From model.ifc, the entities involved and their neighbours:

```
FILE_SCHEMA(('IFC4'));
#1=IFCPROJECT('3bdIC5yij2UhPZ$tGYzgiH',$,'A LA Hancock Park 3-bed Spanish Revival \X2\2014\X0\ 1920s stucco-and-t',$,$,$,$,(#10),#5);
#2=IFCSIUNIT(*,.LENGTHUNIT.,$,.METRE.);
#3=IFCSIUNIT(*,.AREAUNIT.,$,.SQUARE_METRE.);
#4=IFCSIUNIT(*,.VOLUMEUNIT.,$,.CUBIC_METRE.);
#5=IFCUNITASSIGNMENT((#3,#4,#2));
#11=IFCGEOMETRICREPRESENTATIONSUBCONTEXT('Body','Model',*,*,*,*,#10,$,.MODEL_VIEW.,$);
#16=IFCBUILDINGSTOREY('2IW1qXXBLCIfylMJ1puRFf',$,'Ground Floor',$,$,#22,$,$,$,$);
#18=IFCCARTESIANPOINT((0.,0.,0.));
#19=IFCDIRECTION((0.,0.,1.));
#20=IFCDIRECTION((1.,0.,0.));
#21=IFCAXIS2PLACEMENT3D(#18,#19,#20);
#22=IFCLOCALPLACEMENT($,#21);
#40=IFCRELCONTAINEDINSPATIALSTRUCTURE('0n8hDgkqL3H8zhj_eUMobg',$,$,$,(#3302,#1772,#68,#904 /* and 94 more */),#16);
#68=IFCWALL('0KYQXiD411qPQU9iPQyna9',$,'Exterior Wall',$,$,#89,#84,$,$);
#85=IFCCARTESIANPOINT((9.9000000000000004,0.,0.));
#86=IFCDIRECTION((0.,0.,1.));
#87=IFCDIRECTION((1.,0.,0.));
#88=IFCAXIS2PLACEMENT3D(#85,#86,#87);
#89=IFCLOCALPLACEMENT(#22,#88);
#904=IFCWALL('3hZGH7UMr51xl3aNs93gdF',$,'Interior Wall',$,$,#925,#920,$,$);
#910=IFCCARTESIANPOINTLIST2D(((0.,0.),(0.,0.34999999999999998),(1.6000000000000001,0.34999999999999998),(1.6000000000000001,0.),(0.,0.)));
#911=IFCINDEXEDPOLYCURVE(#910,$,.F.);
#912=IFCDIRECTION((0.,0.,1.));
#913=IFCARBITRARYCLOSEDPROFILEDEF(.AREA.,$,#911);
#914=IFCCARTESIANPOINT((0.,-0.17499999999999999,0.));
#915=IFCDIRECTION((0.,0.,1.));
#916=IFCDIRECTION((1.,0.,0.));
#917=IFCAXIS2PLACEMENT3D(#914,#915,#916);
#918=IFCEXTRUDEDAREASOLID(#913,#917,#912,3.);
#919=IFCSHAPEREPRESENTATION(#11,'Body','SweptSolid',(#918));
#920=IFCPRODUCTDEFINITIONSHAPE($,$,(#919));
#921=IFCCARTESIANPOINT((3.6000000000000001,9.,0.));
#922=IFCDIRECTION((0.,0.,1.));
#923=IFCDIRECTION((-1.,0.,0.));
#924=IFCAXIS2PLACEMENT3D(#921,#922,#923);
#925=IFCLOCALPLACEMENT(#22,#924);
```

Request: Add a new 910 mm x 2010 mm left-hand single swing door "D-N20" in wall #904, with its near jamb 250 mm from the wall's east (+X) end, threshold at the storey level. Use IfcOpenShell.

```python
import numpy as np
import ifcopenshell
import ifcopenshell.api.feature
import ifcopenshell.api.geometry
import ifcopenshell.api.root
import ifcopenshell.api.spatial
import ifcopenshell.geom
import ifcopenshell.util.element
import ifcopenshell.util.placement
import ifcopenshell.util.representation
import ifcopenshell.util.shape
import ifcopenshell.util.unit

model = ifcopenshell.open("model.ifc")
unit_scale = ifcopenshell.util.unit.calculate_unit_scale(model)
settings = ifcopenshell.geom.settings()


def volume(element):
    """Net volume in cubic metres, openings subtracted."""
    shape = ifcopenshell.geom.create_shape(settings, element)
    return ifcopenshell.util.shape.get_volume(shape.geometry)


wall = model.by_id(904)
storey = ifcopenshell.util.element.get_container(wall, ifc_class="IfcBuildingStorey")
context = ifcopenshell.util.representation.get_context(model, "Model", "Body", "MODEL_VIEW")
before = volume(wall)

width, height, from_end, sill = 0.91, 2.01, 0.25, 0.0  # metres

# The wall runs along its own X axis, and the end named is its -X end.
wall_shape = ifcopenshell.geom.create_shape(settings, wall)
x, y, z = ifcopenshell.util.shape.get_vertices(wall_shape.geometry).T
start = x.min() + from_end
face, thickness = float(y.min()), float(y.max() - y.min())
wall_matrix = ifcopenshell.util.placement.get_local_placement(wall.ObjectPlacement)
level = ifcopenshell.util.placement.get_local_placement(storey.ObjectPlacement)[2, 3]


def in_wall(x, y):
    """Placement at x, y metres in the wall's axes, at sill height."""
    matrix = wall_matrix.copy()
    matrix[:, 3] = wall_matrix @ np.array([x / unit_scale, y / unit_scale, 0.0, 1.0])
    matrix[2, 3] = level + sill / unit_scale
    return matrix


# Opening: a box that overshoots both wall faces by 50 mm.
opening = ifcopenshell.api.root.create_entity(model, ifc_class="IfcOpeningElement", predefined_type="OPENING")
box = ifcopenshell.api.geometry.add_wall_representation(
    model, context=context, length=width, height=height, thickness=thickness + 0.1
)
ifcopenshell.api.geometry.assign_representation(model, product=opening, representation=box)
ifcopenshell.api.geometry.edit_object_placement(model, product=opening, matrix=in_wall(start, face - 0.05), is_si=False)
ifcopenshell.api.feature.add_feature(model, feature=opening, element=wall)

door = ifcopenshell.api.root.create_entity(model, ifc_class="IfcDoor", name="D-N20", predefined_type="DOOR")
door.OverallWidth, door.OverallHeight = width / unit_scale, height / unit_scale
door.OperationType = "SINGLE_SWING_LEFT"
body = ifcopenshell.api.geometry.add_door_representation(
    model,
    context=context,
    overall_width=door.OverallWidth,
    overall_height=door.OverallHeight,
    operation_type="SINGLE_SWING_LEFT",
    lining_properties={"LiningDepth": thickness / unit_scale, "ThresholdDepth": thickness / unit_scale},
)
ifcopenshell.api.geometry.assign_representation(model, product=door, representation=body)
ifcopenshell.api.spatial.assign_container(model, products=[door], relating_structure=storey)
ifcopenshell.api.feature.add_filling(model, opening=opening, element=door)

# The lining spans the wall, so the door starts at the wall face.
ifcopenshell.api.geometry.edit_object_placement(model, product=door, matrix=in_wall(start, face), is_si=False)

after = volume(wall)

print(f"wall volume {before:.3f} -> {after:.3f} m3")

model.write("model_edited.ifc")
```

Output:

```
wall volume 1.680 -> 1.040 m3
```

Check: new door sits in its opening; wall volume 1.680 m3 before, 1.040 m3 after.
